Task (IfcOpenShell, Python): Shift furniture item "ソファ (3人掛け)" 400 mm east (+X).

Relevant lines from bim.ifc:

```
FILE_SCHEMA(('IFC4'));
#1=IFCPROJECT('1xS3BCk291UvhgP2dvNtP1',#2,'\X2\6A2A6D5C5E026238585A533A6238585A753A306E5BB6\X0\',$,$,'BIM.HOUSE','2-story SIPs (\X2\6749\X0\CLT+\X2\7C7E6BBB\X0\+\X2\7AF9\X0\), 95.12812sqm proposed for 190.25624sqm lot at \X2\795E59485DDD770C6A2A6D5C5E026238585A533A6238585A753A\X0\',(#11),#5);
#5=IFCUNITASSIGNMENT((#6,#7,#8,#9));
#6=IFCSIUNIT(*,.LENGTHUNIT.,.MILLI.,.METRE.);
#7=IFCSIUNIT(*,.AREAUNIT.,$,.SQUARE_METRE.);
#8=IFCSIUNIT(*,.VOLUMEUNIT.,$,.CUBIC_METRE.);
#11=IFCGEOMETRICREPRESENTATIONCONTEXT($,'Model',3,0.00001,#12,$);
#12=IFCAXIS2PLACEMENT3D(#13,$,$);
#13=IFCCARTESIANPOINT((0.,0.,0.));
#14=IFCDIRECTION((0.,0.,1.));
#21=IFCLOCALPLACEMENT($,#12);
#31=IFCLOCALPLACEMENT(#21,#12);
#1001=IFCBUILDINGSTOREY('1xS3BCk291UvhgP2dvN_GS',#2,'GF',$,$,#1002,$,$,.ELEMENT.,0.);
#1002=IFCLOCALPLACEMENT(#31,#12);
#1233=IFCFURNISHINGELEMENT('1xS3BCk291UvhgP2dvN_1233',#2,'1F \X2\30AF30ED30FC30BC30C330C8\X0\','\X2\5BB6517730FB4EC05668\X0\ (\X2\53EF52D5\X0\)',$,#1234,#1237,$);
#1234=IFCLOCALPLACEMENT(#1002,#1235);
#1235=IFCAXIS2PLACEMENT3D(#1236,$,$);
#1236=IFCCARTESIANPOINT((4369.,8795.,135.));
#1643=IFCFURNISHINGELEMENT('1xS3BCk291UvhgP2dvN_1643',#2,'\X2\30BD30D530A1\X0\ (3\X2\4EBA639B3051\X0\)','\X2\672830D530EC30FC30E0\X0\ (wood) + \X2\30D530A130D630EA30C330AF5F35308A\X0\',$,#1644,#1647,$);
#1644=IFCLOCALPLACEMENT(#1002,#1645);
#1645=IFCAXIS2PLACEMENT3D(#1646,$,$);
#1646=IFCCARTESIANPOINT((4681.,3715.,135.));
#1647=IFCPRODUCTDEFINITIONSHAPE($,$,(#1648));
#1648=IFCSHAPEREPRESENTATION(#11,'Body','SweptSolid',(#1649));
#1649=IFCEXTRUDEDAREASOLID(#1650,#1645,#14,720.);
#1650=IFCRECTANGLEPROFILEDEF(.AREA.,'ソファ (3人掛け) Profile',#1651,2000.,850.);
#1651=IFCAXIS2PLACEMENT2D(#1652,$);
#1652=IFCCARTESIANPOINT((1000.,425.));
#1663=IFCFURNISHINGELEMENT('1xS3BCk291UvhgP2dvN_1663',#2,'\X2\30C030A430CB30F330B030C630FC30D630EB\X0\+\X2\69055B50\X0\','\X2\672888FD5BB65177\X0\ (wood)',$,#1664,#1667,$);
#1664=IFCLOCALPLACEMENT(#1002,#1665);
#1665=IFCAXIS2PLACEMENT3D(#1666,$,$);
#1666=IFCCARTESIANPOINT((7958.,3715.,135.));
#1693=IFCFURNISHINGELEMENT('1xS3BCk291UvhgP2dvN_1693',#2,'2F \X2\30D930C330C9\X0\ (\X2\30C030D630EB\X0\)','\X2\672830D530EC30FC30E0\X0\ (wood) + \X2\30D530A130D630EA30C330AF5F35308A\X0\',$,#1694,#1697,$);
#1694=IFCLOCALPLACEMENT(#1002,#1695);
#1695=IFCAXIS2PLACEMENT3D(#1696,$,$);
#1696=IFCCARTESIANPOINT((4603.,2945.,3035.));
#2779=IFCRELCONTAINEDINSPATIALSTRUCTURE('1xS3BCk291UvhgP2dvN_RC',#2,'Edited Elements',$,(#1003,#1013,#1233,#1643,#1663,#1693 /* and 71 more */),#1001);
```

```python
import ifcopenshell
import ifcopenshell.api.geometry
import ifcopenshell.util.placement
import ifcopenshell.util.unit

model = ifcopenshell.open("bim.ifc")
unit_scale = ifcopenshell.util.unit.calculate_unit_scale(model)

item = model.by_guid("1xS3BCk291UvhgP2dvN_1643")
matrix = ifcopenshell.util.placement.get_local_placement(item.ObjectPlacement)
matrix[0, 3] += 0.4 / unit_scale
ifcopenshell.api.geometry.edit_object_placement(model, product=item, matrix=matrix, is_si=False)

print(ifcopenshell.util.placement.get_local_placement(item.ObjectPlacement).round(3) + 0.0)

model.write("bim_edited.ifc")
```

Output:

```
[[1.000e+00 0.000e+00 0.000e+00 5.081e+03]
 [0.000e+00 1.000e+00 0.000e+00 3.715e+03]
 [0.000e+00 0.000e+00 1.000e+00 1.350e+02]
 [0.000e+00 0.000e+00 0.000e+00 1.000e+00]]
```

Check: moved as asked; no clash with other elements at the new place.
